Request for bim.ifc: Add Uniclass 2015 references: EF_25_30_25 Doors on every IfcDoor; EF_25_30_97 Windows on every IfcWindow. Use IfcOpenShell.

First a look at what the model holds.

```python
import ifcopenshell

model = ifcopenshell.open("bim.ifc")
print(model.schema)
print("classifications:", [c.Name for c in model.by_type("IfcClassification")])
for ifc_class in ("IfcDoor", "IfcRoof", "IfcStair", "IfcWall", "IfcWindow"):
    print(ifc_class, len(model.by_type(ifc_class)))
```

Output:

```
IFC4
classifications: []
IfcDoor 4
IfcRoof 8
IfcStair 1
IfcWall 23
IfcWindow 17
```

```python
import ifcopenshell
import ifcopenshell.api.classification

model = ifcopenshell.open("bim.ifc")

system = ifcopenshell.api.classification.add_classification(model, classification="Uniclass 2015")

codes = {
    "IfcDoor": ("EF_25_30_25", "Doors"),
    "IfcWindow": ("EF_25_30_97", "Windows"),
}
for ifc_class, (code, name) in codes.items():
    products = model.by_type(ifc_class)
    ifcopenshell.api.classification.add_reference(
        model, products=products, classification=system, identification=code, name=name
    )
    print(code, len(products))

model.write("bim_rev.ifc")
```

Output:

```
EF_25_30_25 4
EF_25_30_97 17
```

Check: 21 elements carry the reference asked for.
